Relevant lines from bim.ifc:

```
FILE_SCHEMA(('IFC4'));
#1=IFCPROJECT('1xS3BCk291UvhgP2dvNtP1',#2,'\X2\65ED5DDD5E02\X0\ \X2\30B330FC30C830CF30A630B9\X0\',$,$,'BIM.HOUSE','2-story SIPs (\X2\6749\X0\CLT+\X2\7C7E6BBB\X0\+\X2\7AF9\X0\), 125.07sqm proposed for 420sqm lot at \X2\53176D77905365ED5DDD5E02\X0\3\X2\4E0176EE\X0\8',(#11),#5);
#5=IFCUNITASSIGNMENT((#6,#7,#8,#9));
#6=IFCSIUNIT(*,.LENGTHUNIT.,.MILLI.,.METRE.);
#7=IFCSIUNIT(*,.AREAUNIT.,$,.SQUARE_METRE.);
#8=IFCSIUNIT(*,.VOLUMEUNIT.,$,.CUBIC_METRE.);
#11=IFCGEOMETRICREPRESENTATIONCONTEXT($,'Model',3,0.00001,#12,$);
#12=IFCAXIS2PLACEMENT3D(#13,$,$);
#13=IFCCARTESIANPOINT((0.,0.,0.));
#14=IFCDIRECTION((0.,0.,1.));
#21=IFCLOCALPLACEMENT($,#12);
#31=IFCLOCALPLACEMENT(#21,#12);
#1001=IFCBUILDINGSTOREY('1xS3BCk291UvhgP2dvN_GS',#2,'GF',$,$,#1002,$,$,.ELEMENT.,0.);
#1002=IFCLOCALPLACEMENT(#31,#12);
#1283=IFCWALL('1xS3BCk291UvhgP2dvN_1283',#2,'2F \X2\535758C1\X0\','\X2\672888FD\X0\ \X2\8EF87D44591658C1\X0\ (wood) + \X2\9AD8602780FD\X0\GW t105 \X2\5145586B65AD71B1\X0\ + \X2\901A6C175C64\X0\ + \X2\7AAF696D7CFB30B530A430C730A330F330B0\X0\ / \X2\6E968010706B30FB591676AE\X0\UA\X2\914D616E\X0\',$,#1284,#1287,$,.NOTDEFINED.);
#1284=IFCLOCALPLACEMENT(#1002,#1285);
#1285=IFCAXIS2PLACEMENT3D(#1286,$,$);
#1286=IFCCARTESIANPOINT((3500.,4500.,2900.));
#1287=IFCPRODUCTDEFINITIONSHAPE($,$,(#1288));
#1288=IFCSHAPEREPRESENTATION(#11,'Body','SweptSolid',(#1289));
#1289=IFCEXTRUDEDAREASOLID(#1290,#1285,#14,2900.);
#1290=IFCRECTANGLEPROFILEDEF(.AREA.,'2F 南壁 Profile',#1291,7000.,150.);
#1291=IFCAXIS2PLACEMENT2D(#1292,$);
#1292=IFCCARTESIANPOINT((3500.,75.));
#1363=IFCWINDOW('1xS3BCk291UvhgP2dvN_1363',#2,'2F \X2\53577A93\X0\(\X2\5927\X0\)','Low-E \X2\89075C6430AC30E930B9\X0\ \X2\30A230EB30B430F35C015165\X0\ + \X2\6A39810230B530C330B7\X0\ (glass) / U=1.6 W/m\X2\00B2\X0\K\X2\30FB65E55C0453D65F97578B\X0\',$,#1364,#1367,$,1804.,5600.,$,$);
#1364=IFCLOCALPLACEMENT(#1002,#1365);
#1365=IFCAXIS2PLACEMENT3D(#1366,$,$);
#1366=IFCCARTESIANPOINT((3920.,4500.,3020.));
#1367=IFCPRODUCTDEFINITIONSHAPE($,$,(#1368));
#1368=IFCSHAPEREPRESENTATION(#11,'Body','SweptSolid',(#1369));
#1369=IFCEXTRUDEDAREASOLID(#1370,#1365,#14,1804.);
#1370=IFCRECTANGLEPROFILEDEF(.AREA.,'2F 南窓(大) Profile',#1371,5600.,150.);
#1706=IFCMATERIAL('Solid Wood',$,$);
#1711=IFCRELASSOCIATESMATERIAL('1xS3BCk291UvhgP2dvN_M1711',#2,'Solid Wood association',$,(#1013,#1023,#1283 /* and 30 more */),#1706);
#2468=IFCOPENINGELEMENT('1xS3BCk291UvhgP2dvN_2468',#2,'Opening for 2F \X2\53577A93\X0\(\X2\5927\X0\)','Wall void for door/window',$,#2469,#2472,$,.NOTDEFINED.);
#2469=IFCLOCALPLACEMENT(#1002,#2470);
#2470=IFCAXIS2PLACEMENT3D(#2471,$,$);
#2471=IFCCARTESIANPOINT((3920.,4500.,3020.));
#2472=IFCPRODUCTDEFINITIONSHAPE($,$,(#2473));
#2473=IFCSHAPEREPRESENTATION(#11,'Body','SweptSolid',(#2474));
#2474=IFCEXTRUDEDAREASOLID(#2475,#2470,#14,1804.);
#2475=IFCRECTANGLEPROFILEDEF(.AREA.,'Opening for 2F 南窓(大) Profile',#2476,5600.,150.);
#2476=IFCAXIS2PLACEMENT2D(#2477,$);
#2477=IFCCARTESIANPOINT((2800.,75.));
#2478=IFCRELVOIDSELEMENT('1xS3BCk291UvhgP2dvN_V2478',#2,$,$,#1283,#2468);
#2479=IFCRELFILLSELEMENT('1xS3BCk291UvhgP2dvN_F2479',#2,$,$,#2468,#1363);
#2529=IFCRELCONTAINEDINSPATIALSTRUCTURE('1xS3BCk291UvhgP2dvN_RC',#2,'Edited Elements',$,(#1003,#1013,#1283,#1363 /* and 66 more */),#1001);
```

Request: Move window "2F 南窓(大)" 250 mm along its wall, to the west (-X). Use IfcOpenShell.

```python
import ifcopenshell
import ifcopenshell.api.geometry
import ifcopenshell.util.placement
import ifcopenshell.util.unit

model = ifcopenshell.open("bim.ifc")
unit_scale = ifcopenshell.util.unit.calculate_unit_scale(model)

window = model.by_guid("1xS3BCk291UvhgP2dvN_1363")
opening = window.FillsVoids[0].RelatingOpeningElement
wall = opening.VoidsElements[0].RelatingBuildingElement

wall_matrix = ifcopenshell.util.placement.get_local_placement(wall.ObjectPlacement)
shift = wall_matrix[:3, 0] * -0.25 / unit_scale
before = ifcopenshell.util.placement.get_local_placement(window.ObjectPlacement)[:3, 3].copy()

# The window is not placed relative to its opening, so move both.
for product in (opening, window):
    matrix = ifcopenshell.util.placement.get_local_placement(product.ObjectPlacement)
    matrix[:3, 3] += shift
    ifcopenshell.api.geometry.edit_object_placement(model, product=product, matrix=matrix, is_si=False)

after = ifcopenshell.util.placement.get_local_placement(window.ObjectPlacement)[:3, 3]
print("window moved by", (after - before).round(3) + 0.0)

model.write("bim_edited.ifc")
```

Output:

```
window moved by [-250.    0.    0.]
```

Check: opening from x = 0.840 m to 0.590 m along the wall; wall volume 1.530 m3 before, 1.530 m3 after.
